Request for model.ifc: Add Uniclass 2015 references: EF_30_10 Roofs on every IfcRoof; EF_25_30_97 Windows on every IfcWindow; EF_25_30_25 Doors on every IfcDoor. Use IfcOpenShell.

First a look at what the model holds.

```python
import ifcopenshell

model = ifcopenshell.open("model.ifc")
print(model.schema)
print("classifications:", [c.Name for c in model.by_type("IfcClassification")])
for ifc_class in ("IfcDoor", "IfcRoof", "IfcStair", "IfcWall", "IfcWindow"):
    print(ifc_class, len(model.by_type(ifc_class)))
```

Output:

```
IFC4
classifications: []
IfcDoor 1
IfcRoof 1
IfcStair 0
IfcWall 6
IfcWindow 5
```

```python
import ifcopenshell
import ifcopenshell.api.classification

model = ifcopenshell.open("model.ifc")

system = ifcopenshell.api.classification.add_classification(model, classification="Uniclass 2015")

codes = {
    "IfcRoof": ("EF_30_10", "Roofs"),
    "IfcWindow": ("EF_25_30_97", "Windows"),
    "IfcDoor": ("EF_25_30_25", "Doors"),
}
for ifc_class, (code, name) in codes.items():
    products = model.by_type(ifc_class)
    ifcopenshell.api.classification.add_reference(
        model, products=products, classification=system, identification=code, name=name
    )
    print(code, len(products))

model.write("model_v2.ifc")
```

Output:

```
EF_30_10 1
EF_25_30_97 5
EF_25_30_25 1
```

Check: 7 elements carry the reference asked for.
